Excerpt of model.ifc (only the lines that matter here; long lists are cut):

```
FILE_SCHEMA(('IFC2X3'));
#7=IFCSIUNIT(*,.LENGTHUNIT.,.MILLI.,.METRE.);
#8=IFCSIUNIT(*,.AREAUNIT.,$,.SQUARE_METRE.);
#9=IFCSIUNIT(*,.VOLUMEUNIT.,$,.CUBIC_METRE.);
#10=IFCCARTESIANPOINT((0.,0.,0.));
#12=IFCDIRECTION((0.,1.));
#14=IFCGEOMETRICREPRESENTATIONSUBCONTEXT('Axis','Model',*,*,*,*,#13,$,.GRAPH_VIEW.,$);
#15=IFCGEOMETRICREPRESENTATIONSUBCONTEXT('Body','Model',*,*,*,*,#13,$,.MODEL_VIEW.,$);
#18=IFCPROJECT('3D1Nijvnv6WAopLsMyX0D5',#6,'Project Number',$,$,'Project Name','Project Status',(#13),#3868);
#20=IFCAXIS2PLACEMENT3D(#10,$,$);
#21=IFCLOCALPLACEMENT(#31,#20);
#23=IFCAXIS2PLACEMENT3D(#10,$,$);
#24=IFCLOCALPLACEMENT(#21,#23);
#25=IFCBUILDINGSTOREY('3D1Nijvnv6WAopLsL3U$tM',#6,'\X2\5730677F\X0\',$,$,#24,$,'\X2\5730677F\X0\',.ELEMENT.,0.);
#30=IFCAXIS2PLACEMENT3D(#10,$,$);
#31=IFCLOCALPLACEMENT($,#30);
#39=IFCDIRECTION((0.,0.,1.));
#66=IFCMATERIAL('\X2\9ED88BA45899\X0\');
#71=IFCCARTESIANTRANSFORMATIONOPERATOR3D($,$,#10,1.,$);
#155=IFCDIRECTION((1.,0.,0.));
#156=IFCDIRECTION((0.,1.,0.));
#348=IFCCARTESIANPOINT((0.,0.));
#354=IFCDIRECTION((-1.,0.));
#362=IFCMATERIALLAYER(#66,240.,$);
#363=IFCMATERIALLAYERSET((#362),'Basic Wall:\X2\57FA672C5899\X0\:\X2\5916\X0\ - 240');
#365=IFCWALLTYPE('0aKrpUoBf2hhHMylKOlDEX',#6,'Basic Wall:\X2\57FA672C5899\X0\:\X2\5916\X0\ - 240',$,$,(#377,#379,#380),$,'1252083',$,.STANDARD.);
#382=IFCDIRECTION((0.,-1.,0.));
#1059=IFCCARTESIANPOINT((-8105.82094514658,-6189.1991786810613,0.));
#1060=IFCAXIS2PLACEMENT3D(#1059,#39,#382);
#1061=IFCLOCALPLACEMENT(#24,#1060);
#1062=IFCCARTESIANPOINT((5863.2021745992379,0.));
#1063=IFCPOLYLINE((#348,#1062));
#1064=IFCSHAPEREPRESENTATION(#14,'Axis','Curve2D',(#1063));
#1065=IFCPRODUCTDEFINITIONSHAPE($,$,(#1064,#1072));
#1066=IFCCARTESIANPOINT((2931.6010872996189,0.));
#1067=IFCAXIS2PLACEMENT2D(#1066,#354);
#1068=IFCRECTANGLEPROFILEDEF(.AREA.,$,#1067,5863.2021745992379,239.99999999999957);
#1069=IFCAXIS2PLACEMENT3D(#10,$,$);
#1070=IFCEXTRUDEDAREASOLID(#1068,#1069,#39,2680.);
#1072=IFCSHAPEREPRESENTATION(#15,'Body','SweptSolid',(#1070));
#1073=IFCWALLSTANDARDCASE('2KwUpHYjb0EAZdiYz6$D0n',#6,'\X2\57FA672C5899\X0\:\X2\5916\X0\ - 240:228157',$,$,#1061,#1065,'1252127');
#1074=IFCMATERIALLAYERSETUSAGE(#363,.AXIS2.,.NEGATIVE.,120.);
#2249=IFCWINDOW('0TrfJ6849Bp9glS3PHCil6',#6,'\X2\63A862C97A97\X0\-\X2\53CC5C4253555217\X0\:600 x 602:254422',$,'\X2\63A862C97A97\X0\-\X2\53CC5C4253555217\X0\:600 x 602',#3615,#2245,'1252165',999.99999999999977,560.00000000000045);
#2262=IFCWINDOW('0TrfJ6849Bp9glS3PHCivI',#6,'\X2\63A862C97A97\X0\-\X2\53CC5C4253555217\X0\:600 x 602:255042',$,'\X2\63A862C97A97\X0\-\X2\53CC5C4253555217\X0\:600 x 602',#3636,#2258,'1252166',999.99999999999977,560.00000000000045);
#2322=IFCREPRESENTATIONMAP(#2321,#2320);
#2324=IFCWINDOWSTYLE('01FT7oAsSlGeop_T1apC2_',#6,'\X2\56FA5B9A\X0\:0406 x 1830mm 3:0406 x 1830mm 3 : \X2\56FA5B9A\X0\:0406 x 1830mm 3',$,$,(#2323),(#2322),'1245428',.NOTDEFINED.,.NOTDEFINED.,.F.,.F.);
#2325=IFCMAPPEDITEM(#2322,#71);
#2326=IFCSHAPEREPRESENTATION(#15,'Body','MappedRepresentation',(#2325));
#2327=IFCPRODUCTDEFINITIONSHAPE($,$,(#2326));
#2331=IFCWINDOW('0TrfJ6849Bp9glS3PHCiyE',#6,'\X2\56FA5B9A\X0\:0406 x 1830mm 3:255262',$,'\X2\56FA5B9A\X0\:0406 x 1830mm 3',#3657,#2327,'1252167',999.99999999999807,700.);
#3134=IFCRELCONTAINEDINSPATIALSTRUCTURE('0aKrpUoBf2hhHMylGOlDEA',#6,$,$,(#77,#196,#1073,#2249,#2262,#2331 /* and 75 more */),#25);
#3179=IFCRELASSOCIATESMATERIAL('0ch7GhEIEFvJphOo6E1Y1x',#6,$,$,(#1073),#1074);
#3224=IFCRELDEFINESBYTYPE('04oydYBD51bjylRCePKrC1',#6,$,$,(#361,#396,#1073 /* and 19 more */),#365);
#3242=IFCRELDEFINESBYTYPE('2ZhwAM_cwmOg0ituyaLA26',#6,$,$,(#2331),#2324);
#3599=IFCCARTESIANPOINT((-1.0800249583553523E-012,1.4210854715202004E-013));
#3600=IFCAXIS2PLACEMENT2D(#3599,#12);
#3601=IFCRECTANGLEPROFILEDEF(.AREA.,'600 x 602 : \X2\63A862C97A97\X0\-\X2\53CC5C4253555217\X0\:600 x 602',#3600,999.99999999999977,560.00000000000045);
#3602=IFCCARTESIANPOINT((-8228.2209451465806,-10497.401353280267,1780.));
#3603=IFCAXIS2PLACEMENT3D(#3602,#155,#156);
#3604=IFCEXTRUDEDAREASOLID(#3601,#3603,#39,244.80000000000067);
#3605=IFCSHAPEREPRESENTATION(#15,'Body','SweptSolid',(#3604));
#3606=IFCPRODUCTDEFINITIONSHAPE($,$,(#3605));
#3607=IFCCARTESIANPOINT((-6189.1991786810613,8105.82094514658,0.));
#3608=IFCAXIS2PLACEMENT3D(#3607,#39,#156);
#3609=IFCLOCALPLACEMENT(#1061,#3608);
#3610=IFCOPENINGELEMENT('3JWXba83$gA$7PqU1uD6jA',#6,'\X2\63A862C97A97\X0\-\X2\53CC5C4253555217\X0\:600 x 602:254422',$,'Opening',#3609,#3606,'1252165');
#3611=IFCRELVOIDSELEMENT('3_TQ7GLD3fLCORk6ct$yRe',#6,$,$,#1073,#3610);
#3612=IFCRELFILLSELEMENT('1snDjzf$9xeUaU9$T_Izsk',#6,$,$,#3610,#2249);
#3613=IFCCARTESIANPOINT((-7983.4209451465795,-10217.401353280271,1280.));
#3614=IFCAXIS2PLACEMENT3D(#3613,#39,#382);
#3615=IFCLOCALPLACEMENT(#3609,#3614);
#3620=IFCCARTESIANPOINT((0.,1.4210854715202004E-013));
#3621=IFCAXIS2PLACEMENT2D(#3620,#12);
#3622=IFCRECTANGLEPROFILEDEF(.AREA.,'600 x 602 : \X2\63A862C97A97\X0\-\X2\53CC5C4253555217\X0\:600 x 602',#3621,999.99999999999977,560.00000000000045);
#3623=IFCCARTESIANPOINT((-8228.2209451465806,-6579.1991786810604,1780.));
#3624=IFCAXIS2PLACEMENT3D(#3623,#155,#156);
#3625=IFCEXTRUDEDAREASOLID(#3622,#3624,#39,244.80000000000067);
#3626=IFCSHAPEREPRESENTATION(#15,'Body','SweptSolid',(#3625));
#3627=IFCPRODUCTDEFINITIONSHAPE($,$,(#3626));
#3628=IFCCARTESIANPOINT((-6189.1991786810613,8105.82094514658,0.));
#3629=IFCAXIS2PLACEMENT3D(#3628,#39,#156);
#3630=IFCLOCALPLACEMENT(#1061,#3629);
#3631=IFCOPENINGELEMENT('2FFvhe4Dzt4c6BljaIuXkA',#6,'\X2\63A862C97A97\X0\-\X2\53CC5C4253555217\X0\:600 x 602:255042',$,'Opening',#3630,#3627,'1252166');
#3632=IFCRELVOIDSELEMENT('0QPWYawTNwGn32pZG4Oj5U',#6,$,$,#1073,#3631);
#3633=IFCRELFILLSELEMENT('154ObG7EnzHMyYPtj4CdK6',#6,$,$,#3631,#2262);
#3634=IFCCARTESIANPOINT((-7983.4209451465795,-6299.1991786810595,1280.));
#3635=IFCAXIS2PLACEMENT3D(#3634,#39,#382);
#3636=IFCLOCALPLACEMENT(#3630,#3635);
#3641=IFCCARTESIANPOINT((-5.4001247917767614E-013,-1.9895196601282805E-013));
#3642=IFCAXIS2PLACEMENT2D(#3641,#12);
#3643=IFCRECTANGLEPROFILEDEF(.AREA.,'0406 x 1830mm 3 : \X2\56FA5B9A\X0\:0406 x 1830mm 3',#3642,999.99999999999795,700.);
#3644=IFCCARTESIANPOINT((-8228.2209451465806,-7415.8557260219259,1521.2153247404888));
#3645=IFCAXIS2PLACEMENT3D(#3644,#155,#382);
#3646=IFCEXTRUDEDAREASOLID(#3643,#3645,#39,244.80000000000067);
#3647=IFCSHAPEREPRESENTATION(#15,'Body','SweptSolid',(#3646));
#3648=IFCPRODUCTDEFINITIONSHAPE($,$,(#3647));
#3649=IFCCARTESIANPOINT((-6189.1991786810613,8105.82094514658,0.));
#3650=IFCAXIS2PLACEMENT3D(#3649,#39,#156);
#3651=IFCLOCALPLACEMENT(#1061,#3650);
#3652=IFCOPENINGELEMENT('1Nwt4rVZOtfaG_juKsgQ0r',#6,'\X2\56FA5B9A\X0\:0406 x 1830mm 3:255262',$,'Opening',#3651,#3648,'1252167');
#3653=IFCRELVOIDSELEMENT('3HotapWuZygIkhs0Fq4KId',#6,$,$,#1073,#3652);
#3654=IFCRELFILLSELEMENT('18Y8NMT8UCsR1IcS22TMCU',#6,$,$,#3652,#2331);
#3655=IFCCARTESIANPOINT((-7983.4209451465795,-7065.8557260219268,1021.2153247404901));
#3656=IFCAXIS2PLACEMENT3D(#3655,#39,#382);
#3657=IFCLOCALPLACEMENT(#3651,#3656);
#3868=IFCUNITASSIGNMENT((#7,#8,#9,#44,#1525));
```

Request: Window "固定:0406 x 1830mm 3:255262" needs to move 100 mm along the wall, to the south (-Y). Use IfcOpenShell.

```python
import ifcopenshell
import ifcopenshell.api.geometry
import ifcopenshell.util.placement
import ifcopenshell.util.unit

model = ifcopenshell.open("model.ifc")
unit_scale = ifcopenshell.util.unit.calculate_unit_scale(model)

window = model.by_id(2331)
opening = window.FillsVoids[0].RelatingOpeningElement
wall = opening.VoidsElements[0].RelatingBuildingElement

wall_matrix = ifcopenshell.util.placement.get_local_placement(wall.ObjectPlacement)
shift = wall_matrix[:3, 0] * 0.1 / unit_scale
before = ifcopenshell.util.placement.get_local_placement(window.ObjectPlacement)[:3, 3].copy()

# The window is placed relative to its opening, so it follows when the opening moves.
matrix = ifcopenshell.util.placement.get_local_placement(opening.ObjectPlacement)
matrix[:3, 3] += shift
ifcopenshell.api.geometry.edit_object_placement(
    model, product=opening, matrix=matrix, is_si=False, should_transform_children=True
)

after = ifcopenshell.util.placement.get_local_placement(window.ObjectPlacement)[:3, 3]
print("window moved by", (after - before).round(3) + 0.0)

model.write("model-out.ifc")
```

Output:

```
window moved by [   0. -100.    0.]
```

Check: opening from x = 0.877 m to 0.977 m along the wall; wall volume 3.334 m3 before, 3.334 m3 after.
